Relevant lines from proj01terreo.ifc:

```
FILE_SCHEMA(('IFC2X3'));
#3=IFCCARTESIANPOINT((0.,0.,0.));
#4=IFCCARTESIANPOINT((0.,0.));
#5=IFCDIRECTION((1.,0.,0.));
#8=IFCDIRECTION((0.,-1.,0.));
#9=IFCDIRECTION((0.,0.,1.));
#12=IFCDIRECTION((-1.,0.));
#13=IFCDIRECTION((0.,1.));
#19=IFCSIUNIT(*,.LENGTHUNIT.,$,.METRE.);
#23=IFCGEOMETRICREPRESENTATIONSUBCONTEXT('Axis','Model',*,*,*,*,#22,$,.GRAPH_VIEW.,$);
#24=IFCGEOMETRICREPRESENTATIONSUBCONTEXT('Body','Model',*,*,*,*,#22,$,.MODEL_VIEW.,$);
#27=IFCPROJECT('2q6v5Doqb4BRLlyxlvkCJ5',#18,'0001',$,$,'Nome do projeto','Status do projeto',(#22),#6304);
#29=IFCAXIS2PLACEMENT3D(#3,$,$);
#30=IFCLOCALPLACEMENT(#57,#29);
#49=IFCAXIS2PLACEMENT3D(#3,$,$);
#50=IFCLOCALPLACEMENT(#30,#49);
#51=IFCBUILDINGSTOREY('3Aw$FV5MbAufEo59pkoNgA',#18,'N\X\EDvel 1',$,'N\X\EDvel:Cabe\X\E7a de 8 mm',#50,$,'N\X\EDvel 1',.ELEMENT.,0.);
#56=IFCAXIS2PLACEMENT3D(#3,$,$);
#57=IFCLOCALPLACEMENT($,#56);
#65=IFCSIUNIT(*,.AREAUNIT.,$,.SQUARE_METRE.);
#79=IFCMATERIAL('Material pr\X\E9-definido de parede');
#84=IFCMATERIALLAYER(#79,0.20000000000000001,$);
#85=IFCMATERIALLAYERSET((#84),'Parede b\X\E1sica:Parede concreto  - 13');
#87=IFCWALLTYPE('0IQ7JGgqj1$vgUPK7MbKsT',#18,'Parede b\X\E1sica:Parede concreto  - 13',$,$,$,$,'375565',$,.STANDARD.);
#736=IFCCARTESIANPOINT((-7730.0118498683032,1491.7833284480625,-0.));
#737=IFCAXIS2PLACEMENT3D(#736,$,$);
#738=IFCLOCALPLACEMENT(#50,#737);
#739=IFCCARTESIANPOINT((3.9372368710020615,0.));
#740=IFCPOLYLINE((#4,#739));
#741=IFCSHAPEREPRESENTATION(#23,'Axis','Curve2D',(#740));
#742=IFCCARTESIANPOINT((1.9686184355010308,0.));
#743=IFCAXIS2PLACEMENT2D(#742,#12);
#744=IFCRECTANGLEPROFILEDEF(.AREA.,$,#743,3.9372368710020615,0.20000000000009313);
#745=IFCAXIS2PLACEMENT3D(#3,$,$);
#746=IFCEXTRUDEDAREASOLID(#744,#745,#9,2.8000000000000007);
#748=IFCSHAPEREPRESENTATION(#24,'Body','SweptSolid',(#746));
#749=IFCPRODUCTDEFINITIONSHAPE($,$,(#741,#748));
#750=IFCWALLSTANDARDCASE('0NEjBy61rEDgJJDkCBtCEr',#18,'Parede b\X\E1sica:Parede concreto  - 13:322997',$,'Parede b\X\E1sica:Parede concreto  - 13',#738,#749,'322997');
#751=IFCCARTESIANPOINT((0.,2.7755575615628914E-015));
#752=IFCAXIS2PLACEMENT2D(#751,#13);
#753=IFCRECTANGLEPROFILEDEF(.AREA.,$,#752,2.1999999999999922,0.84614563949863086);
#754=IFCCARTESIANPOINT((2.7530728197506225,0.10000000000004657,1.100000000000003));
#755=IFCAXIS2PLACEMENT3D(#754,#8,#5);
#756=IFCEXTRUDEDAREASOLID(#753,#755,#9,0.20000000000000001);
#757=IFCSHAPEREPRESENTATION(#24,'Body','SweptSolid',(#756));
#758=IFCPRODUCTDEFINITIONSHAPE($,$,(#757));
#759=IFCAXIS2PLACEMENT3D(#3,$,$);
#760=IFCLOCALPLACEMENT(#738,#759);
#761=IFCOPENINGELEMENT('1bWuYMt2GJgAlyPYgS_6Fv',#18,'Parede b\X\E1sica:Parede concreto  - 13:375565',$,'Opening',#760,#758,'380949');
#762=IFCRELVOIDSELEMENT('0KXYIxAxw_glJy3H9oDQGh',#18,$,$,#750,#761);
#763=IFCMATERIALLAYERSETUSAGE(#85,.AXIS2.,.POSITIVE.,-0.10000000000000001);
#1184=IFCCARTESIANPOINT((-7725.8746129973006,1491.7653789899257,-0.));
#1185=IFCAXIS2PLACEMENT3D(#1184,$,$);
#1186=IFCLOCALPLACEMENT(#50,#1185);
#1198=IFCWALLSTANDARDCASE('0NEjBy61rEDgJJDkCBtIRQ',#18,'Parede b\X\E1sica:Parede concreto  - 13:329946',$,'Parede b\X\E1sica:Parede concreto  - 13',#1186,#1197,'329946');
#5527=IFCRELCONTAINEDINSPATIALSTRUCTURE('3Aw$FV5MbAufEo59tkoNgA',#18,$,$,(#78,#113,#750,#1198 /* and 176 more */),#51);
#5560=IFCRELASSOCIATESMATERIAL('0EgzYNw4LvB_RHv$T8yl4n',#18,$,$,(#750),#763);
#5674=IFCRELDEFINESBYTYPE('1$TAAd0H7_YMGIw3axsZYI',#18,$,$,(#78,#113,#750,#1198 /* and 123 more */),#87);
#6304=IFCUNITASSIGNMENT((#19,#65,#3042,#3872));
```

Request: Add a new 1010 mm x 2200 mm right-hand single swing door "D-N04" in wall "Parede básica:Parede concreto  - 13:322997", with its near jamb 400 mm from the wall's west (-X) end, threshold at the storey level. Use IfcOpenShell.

```python
import numpy as np
import ifcopenshell
import ifcopenshell.api.feature
import ifcopenshell.api.geometry
import ifcopenshell.api.root
import ifcopenshell.api.spatial
import ifcopenshell.api.type
import ifcopenshell.geom
import ifcopenshell.util.element
import ifcopenshell.util.placement
import ifcopenshell.util.representation
import ifcopenshell.util.shape
import ifcopenshell.util.unit

model = ifcopenshell.open("proj01terreo.ifc")
unit_scale = ifcopenshell.util.unit.calculate_unit_scale(model)
settings = ifcopenshell.geom.settings()


def volume(element):
    """Net volume in cubic metres, openings subtracted."""
    shape = ifcopenshell.geom.create_shape(settings, element)
    return ifcopenshell.util.shape.get_volume(shape.geometry)


wall = model.by_guid("0NEjBy61rEDgJJDkCBtCEr")
storey = ifcopenshell.util.element.get_container(wall, ifc_class="IfcBuildingStorey")
context = ifcopenshell.util.representation.get_context(model, "Model", "Body", "MODEL_VIEW")
before = volume(wall)

width, height, from_end, sill = 1.01, 2.2, 0.4, 0.0  # metres

# The wall runs along its own X axis, and the end named is its -X end.
wall_shape = ifcopenshell.geom.create_shape(settings, wall)
x, y, z = ifcopenshell.util.shape.get_vertices(wall_shape.geometry).T
start = x.min() + from_end
face, thickness = float(y.min()), float(y.max() - y.min())
wall_matrix = ifcopenshell.util.placement.get_local_placement(wall.ObjectPlacement)
level = ifcopenshell.util.placement.get_local_placement(storey.ObjectPlacement)[2, 3]


def in_wall(x, y):
    """Placement at x, y metres in the wall's axes, at sill height."""
    matrix = wall_matrix.copy()
    matrix[:, 3] = wall_matrix @ np.array([x / unit_scale, y / unit_scale, 0.0, 1.0])
    matrix[2, 3] = level + sill / unit_scale
    return matrix


# Opening: a box that overshoots both wall faces by 50 mm.
opening = ifcopenshell.api.root.create_entity(model, ifc_class="IfcOpeningElement")
box = ifcopenshell.api.geometry.add_wall_representation(
    model, context=context, length=width, height=height, thickness=thickness + 0.1
)
ifcopenshell.api.geometry.assign_representation(model, product=opening, representation=box)
ifcopenshell.api.geometry.edit_object_placement(model, product=opening, matrix=in_wall(start, face - 0.05), is_si=False)
ifcopenshell.api.feature.add_feature(model, feature=opening, element=wall)

door = ifcopenshell.api.root.create_entity(model, ifc_class="IfcDoor", name="D-N04")
door.OverallWidth, door.OverallHeight = width / unit_scale, height / unit_scale
body = ifcopenshell.api.geometry.add_door_representation(
    model,
    context=context,
    overall_width=door.OverallWidth,
    overall_height=door.OverallHeight,
    operation_type="SINGLE_SWING_RIGHT",
    lining_properties={"LiningDepth": thickness / unit_scale, "ThresholdDepth": thickness / unit_scale},
)
ifcopenshell.api.geometry.assign_representation(model, product=door, representation=body)
ifcopenshell.api.spatial.assign_container(model, products=[door], relating_structure=storey)
fills = ifcopenshell.api.feature.add_filling(model, opening=opening, element=door)
fills.OwnerHistory = door.OwnerHistory  # required in IFC2X3

# IFC2X3 keeps the operation on the door style.
style = ifcopenshell.api.root.create_entity(model, ifc_class="IfcDoorStyle", name="D-N04")
style.OperationType, style.ConstructionType = "SINGLE_SWING_RIGHT", "NOTDEFINED"
style.ParameterTakesPrecedence = style.Sizeable = False
ifcopenshell.api.type.assign_type(model, related_objects=[door], relating_type=style)

# The lining spans the wall, so the door starts at the wall face.
ifcopenshell.api.geometry.edit_object_placement(model, product=door, matrix=in_wall(start, face), is_si=False)

after = volume(wall)

print(f"wall volume {before:.3f} -> {after:.3f} m3")

model.write("proj01terreo_rev.ifc")
```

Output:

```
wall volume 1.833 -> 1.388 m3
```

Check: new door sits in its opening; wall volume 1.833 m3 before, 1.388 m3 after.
